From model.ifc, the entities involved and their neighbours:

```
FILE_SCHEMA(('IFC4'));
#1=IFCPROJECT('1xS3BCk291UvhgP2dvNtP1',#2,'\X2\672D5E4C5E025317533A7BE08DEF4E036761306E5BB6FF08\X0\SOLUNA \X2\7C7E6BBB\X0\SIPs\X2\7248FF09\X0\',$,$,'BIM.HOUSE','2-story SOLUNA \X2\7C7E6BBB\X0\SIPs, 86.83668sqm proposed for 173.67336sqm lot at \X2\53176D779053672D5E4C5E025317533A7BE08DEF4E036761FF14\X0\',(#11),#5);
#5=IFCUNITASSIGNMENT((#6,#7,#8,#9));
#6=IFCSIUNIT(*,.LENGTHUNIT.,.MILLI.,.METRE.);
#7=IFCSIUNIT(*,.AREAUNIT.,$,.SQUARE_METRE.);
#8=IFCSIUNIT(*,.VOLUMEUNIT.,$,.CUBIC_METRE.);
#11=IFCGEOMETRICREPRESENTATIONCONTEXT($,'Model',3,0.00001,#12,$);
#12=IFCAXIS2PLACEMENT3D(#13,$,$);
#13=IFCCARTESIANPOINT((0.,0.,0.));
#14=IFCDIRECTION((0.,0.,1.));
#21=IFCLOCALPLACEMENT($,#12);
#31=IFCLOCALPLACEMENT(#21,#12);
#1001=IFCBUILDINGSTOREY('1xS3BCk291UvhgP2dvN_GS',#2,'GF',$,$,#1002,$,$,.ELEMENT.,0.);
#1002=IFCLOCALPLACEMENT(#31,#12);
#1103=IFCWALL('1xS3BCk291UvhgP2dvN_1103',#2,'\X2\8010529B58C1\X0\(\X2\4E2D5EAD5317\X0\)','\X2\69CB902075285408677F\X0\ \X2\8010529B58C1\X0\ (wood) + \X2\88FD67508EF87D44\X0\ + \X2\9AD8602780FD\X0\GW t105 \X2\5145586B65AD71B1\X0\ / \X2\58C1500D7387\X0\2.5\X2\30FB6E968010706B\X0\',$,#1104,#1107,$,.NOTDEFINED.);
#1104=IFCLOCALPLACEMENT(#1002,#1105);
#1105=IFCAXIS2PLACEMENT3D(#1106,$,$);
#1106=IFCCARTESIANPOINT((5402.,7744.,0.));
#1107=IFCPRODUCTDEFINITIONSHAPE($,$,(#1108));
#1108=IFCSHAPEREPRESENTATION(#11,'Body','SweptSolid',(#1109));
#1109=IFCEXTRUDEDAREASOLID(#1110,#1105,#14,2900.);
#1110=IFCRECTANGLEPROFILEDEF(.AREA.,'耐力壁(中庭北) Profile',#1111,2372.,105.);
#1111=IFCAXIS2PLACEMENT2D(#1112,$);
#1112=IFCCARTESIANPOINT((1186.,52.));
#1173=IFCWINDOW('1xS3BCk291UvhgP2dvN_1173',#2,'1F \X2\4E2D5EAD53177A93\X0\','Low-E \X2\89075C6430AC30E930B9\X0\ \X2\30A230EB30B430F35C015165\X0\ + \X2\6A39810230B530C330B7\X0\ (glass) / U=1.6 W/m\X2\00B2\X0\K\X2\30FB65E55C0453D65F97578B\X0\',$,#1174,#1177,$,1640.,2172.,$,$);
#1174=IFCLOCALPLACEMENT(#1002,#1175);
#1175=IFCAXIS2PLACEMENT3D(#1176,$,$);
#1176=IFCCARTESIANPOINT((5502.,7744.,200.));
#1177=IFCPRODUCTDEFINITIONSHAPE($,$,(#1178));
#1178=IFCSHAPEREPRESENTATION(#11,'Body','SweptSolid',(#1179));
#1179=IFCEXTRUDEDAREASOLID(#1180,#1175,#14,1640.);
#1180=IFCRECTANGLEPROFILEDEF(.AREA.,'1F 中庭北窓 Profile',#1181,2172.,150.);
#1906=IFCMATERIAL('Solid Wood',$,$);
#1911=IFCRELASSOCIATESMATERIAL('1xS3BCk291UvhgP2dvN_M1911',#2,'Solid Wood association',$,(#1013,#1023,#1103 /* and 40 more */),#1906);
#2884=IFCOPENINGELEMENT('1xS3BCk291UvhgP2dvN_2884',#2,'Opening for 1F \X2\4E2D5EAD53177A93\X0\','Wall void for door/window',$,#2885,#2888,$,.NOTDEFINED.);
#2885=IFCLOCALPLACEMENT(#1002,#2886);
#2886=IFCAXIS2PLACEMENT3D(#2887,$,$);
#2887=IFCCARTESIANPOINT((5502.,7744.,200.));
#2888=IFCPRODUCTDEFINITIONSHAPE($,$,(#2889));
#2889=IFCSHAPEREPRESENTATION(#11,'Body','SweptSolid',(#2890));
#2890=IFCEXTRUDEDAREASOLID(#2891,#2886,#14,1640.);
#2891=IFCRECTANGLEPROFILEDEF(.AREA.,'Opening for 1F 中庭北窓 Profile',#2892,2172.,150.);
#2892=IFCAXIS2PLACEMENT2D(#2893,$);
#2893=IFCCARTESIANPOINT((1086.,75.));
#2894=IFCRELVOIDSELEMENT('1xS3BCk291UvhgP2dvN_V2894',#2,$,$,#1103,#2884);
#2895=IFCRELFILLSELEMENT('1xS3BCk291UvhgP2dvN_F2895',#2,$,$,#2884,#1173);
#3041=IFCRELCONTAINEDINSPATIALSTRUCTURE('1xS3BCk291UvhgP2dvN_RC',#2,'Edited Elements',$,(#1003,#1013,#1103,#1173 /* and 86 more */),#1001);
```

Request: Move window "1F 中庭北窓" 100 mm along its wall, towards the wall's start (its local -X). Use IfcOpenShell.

```python
import ifcopenshell
import ifcopenshell.api.geometry
import ifcopenshell.util.placement
import ifcopenshell.util.unit

model = ifcopenshell.open("model.ifc")
unit_scale = ifcopenshell.util.unit.calculate_unit_scale(model)

window = model.by_guid("1xS3BCk291UvhgP2dvN_1173")
opening = window.FillsVoids[0].RelatingOpeningElement
wall = opening.VoidsElements[0].RelatingBuildingElement

wall_matrix = ifcopenshell.util.placement.get_local_placement(wall.ObjectPlacement)
shift = wall_matrix[:3, 0] * -0.1 / unit_scale
before = ifcopenshell.util.placement.get_local_placement(window.ObjectPlacement)[:3, 3].copy()

# The window is not placed relative to its opening, so move both.
for product in (opening, window):
    matrix = ifcopenshell.util.placement.get_local_placement(product.ObjectPlacement)
    matrix[:3, 3] += shift
    ifcopenshell.api.geometry.edit_object_placement(model, product=product, matrix=matrix, is_si=False)

after = ifcopenshell.util.placement.get_local_placement(window.ObjectPlacement)[:3, 3]
print("window moved by", (after - before).round(3) + 0.0)

model.write("model-out.ifc")
```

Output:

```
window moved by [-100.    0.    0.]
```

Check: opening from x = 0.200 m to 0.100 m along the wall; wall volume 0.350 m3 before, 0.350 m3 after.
